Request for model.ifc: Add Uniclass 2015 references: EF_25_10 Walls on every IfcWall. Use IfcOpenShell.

First a look at what the model holds.

```python
import ifcopenshell

model = ifcopenshell.open("model.ifc")
print(model.schema)
print("classifications:", [c.Name for c in model.by_type("IfcClassification")])
for ifc_class in ("IfcDoor", "IfcRoof", "IfcStair", "IfcWall", "IfcWindow"):
    print(ifc_class, len(model.by_type(ifc_class)))
```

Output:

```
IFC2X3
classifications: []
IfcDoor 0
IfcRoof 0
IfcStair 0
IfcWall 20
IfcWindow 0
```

```python
import ifcopenshell
import ifcopenshell.api.classification

model = ifcopenshell.open("model.ifc")

# IFC2X3 requires Source and Edition and has no link from the project to the system.
system = model.create_entity("IfcClassification", Source="NBS", Edition="2015", Name="Uniclass 2015")

codes = {
    "IfcWall": ("EF_25_10", "Walls"),
}
for ifc_class, (code, name) in codes.items():
    products = model.by_type(ifc_class)
    ifcopenshell.api.classification.add_reference(
        model, products=products, classification=system, identification=code, name=name
    )
    print(code, len(products))

model.write("model_updated.ifc")
```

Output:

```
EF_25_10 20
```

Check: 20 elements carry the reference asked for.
